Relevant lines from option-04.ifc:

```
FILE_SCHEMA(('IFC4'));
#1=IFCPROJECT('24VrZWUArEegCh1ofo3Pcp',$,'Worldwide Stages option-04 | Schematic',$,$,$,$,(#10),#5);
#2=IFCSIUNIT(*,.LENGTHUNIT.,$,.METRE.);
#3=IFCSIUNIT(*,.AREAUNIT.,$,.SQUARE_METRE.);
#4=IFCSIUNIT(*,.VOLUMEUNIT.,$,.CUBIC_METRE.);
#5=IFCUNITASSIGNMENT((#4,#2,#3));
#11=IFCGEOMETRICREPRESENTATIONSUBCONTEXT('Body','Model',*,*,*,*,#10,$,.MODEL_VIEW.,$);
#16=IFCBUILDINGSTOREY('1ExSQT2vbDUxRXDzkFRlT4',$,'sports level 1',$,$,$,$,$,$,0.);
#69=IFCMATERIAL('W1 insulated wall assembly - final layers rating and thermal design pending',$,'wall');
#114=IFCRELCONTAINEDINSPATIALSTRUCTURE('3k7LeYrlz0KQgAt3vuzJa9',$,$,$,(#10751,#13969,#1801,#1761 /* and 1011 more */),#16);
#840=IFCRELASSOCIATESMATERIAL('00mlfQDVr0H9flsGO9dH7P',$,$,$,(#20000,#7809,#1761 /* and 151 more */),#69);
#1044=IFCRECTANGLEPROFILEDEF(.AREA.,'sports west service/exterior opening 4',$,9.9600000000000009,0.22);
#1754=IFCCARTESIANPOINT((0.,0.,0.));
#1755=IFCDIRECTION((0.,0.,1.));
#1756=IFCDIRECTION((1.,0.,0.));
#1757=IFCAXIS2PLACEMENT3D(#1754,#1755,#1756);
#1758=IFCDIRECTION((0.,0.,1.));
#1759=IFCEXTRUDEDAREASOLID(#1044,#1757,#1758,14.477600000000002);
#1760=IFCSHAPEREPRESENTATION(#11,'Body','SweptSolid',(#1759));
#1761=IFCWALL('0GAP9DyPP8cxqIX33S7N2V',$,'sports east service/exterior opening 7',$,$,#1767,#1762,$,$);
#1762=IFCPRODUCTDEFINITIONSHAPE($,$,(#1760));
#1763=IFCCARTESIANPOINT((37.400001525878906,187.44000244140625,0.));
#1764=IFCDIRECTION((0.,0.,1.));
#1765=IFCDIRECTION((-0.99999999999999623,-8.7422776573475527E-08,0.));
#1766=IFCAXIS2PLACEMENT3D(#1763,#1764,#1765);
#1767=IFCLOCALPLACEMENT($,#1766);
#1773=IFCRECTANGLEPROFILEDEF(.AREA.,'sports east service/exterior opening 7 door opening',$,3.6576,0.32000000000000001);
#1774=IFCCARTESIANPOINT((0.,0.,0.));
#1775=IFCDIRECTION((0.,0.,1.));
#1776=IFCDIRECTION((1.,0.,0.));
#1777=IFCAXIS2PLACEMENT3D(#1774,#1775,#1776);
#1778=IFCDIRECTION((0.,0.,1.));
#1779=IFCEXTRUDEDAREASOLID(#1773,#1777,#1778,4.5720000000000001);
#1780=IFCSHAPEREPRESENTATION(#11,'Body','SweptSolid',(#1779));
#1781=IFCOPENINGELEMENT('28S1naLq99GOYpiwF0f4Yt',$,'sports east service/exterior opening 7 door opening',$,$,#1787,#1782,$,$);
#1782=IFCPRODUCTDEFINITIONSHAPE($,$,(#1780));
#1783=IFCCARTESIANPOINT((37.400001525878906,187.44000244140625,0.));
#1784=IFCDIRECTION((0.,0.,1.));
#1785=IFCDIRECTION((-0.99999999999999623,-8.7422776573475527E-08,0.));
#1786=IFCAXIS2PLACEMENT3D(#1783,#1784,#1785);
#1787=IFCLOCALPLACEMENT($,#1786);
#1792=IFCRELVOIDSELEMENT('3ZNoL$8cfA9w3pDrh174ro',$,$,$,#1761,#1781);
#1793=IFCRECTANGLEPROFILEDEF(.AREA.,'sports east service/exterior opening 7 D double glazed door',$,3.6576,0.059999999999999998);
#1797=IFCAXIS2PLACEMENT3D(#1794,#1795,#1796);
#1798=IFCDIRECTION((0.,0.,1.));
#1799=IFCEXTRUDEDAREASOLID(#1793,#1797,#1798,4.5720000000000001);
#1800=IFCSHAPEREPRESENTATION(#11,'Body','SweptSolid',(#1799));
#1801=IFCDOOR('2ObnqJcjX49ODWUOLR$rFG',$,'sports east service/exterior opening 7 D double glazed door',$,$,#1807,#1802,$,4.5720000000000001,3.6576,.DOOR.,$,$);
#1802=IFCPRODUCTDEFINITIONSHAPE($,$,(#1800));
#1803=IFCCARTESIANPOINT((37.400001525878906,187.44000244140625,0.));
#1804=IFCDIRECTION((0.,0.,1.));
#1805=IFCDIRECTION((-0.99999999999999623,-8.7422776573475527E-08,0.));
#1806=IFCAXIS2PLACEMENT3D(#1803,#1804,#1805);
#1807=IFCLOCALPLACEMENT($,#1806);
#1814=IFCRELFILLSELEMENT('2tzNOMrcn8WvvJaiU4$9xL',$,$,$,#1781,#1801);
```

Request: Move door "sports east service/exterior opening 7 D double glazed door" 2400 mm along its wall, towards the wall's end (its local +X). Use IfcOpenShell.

```python
import ifcopenshell
import ifcopenshell.api.geometry
import ifcopenshell.util.placement
import ifcopenshell.util.unit

model = ifcopenshell.open("option-04.ifc")
unit_scale = ifcopenshell.util.unit.calculate_unit_scale(model)

door = model.by_guid("2ObnqJcjX49ODWUOLR$rFG")
opening = door.FillsVoids[0].RelatingOpeningElement
wall = opening.VoidsElements[0].RelatingBuildingElement

wall_matrix = ifcopenshell.util.placement.get_local_placement(wall.ObjectPlacement)
shift = wall_matrix[:3, 0] * 2.4 / unit_scale
before = ifcopenshell.util.placement.get_local_placement(door.ObjectPlacement)[:3, 3].copy()

# The door is not placed relative to its opening, so move both.
for product in (opening, door):
    matrix = ifcopenshell.util.placement.get_local_placement(product.ObjectPlacement)
    matrix[:3, 3] += shift
    ifcopenshell.api.geometry.edit_object_placement(model, product=product, matrix=matrix, is_si=False)

after = ifcopenshell.util.placement.get_local_placement(door.ObjectPlacement)[:3, 3]
print("door moved by", (after - before).round(3) + 0.0)

model.write("option-04_rev.ifc")
```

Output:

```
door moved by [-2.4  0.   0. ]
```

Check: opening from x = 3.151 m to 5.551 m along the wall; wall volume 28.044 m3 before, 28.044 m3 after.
